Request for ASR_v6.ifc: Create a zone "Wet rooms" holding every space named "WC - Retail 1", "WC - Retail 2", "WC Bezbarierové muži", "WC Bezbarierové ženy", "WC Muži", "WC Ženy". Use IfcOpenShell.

First a look at what the model holds.

```python
import ifcopenshell

model = ifcopenshell.open("ASR_v6.ifc")
print(model.schema)
seen = {}
for space in model.by_type("IfcSpace"):
    seen[space.LongName] = seen.get(space.LongName, 0) + 1
for name, count in sorted(seen.items(), key=str):
    print(count, "x", name)
print("zones:", [z.Name for z in model.by_type("IfcZone")][:20])
```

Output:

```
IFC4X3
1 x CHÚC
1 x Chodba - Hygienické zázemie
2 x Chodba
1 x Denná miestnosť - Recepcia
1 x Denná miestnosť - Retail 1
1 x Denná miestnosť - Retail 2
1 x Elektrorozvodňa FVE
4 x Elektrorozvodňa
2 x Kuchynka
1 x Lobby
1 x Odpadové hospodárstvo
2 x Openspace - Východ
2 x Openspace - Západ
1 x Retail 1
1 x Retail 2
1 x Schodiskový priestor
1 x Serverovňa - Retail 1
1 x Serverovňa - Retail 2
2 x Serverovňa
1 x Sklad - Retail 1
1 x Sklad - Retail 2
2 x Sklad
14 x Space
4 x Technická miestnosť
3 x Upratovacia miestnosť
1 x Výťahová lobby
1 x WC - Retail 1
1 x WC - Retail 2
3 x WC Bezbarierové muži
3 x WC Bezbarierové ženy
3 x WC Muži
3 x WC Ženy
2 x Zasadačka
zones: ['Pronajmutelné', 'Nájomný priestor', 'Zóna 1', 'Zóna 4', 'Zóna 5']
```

```python
import ifcopenshell
import ifcopenshell.api.group
import ifcopenshell.api.root

model = ifcopenshell.open("ASR_v6.ifc")

names = {"WC - Retail 1", "WC - Retail 2", "WC Bezbarierové muži", "WC Bezbarierové ženy", "WC Muži", "WC Ženy"}
spaces = [s for s in model.by_type("IfcSpace") if s.LongName in names]

zone = ifcopenshell.api.root.create_entity(model, ifc_class="IfcZone", name="Wet rooms")
ifcopenshell.api.group.assign_group(model, products=spaces, group=zone)
print(len(spaces), "spaces in", zone.Name)

model.write("ASR_v6-out.ifc")
```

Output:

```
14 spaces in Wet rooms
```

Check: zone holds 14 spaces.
